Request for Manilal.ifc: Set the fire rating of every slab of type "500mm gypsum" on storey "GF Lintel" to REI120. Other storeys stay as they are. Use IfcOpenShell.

First a look at what the model holds.

```python
import ifcopenshell
import ifcopenshell.util.element

model = ifcopenshell.open("Manilal.ifc")
print(model.schema)
storey = next(s for s in model.by_type("IfcBuildingStorey") if s.Name == "GF Lintel")
slabs = [e for e in ifcopenshell.util.element.get_decomposition(storey) if e.is_a("IfcSlab")]
seen = {}
for e in slabs:
    element_type = ifcopenshell.util.element.get_type(e)
    key = (element_type.Name if element_type != e and element_type else None, ifcopenshell.util.element.get_pset(e, "Pset_SlabCommon", "FireRating"))
    seen[key] = seen.get(key, 0) + 1
for (name, value), count in sorted(seen.items(), key=str):
    print(count, "x", name, "|", value)
```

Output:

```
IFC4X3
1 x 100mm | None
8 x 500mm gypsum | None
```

```python
import ifcopenshell
import ifcopenshell.api.pset
import ifcopenshell.util.element

model = ifcopenshell.open("Manilal.ifc")

storey = next(s for s in model.by_type("IfcBuildingStorey") if s.Name == "GF Lintel")
slabs = [e for e in ifcopenshell.util.element.get_decomposition(storey) if e.is_a("IfcSlab")]

count = 0
for e in slabs:
    element_type = ifcopenshell.util.element.get_type(e)
    if element_type in (None, e) or element_type.Name != "500mm gypsum":
        continue
    # add_pset returns the element's existing set when there is one.
    pset = ifcopenshell.api.pset.add_pset(model, product=e, name="Pset_SlabCommon")
    ifcopenshell.api.pset.edit_pset(model, pset=pset, properties={"FireRating": "REI120"})
    count += 1

print(count, "slabs updated")

model.write("Manilal_edited.ifc")
```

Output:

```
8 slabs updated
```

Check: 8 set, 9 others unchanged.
